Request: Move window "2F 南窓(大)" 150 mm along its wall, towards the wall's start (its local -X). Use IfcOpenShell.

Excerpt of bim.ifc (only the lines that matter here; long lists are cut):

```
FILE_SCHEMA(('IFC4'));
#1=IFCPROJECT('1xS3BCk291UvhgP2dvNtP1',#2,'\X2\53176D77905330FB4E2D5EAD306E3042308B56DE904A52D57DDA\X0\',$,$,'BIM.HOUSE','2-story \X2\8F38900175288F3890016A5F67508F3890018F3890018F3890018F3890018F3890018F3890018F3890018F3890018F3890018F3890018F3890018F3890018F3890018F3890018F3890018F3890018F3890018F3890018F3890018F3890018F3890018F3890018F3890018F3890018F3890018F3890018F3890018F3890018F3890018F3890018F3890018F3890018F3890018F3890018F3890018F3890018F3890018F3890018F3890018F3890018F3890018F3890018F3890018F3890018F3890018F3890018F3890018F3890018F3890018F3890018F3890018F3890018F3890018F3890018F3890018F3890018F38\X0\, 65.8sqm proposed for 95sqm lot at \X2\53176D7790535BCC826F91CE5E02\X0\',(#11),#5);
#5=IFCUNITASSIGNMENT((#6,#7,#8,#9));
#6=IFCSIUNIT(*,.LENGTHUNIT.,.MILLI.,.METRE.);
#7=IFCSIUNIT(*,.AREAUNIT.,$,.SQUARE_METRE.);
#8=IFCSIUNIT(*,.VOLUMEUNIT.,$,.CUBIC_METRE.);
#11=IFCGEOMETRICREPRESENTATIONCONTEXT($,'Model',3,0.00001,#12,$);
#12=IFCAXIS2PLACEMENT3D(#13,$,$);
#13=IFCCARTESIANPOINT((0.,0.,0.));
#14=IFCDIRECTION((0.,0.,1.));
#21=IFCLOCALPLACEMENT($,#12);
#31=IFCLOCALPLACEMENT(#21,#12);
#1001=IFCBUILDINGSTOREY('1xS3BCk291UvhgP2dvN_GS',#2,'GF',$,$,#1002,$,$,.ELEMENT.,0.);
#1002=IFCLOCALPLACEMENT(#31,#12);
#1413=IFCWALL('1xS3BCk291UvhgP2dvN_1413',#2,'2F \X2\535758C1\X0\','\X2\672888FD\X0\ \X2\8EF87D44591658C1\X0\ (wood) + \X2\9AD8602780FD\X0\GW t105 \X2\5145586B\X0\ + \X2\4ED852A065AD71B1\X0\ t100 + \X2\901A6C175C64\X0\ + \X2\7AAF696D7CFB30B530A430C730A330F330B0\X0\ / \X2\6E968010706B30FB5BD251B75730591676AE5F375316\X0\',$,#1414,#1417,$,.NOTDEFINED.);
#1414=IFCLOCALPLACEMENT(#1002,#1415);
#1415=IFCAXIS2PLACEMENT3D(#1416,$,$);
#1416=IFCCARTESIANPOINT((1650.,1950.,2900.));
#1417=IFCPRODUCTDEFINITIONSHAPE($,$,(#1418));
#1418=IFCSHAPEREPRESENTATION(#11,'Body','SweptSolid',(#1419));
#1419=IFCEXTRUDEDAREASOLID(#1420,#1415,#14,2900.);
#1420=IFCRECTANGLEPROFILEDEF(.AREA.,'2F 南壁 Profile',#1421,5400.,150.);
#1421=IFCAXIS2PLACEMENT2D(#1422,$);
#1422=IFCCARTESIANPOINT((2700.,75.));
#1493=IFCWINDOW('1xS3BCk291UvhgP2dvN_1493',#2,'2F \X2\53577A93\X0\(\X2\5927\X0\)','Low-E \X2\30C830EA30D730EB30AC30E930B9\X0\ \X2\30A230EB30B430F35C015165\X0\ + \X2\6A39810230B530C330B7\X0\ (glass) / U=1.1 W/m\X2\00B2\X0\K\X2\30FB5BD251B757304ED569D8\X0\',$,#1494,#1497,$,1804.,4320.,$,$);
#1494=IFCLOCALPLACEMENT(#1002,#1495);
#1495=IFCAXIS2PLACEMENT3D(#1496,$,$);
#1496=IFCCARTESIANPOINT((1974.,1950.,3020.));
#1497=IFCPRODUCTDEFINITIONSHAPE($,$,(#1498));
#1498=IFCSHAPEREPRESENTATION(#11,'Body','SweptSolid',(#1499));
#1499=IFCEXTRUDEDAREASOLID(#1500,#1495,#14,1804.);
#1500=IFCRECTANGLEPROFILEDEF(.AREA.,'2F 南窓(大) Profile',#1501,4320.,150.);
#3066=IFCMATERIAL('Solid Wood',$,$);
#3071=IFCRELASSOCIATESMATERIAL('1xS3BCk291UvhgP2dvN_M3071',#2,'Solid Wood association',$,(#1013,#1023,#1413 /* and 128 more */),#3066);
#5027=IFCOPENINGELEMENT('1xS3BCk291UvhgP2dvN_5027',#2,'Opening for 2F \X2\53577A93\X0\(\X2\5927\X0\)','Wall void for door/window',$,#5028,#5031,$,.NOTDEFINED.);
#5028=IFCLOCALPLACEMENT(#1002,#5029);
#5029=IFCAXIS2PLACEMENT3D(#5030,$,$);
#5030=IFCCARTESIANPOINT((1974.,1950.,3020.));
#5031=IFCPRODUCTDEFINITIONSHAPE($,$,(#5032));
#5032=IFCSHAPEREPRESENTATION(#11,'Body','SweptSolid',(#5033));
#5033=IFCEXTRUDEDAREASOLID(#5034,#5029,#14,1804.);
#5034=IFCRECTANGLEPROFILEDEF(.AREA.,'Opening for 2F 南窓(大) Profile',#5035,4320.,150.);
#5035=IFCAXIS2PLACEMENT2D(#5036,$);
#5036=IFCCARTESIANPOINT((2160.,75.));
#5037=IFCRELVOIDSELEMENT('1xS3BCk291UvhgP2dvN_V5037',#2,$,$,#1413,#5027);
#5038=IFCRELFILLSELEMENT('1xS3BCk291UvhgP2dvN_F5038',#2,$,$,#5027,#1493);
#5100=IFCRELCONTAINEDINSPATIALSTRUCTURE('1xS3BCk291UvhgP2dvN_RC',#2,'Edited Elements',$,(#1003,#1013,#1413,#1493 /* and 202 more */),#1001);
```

```python
import ifcopenshell
import ifcopenshell.api.geometry
import ifcopenshell.util.placement
import ifcopenshell.util.unit

model = ifcopenshell.open("bim.ifc")
unit_scale = ifcopenshell.util.unit.calculate_unit_scale(model)

window = model.by_guid("1xS3BCk291UvhgP2dvN_1493")
opening = window.FillsVoids[0].RelatingOpeningElement
wall = opening.VoidsElements[0].RelatingBuildingElement

wall_matrix = ifcopenshell.util.placement.get_local_placement(wall.ObjectPlacement)
shift = wall_matrix[:3, 0] * -0.15 / unit_scale
before = ifcopenshell.util.placement.get_local_placement(window.ObjectPlacement)[:3, 3].copy()

# The window is not placed relative to its opening, so move both.
for product in (opening, window):
    matrix = ifcopenshell.util.placement.get_local_placement(product.ObjectPlacement)
    matrix[:3, 3] += shift
    ifcopenshell.api.geometry.edit_object_placement(model, product=product, matrix=matrix, is_si=False)

after = ifcopenshell.util.placement.get_local_placement(window.ObjectPlacement)[:3, 3]
print("window moved by", (after - before).round(3) + 0.0)

model.write("bim_updated.ifc")
```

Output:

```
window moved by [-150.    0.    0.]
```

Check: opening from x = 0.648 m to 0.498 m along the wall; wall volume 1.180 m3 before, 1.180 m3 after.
